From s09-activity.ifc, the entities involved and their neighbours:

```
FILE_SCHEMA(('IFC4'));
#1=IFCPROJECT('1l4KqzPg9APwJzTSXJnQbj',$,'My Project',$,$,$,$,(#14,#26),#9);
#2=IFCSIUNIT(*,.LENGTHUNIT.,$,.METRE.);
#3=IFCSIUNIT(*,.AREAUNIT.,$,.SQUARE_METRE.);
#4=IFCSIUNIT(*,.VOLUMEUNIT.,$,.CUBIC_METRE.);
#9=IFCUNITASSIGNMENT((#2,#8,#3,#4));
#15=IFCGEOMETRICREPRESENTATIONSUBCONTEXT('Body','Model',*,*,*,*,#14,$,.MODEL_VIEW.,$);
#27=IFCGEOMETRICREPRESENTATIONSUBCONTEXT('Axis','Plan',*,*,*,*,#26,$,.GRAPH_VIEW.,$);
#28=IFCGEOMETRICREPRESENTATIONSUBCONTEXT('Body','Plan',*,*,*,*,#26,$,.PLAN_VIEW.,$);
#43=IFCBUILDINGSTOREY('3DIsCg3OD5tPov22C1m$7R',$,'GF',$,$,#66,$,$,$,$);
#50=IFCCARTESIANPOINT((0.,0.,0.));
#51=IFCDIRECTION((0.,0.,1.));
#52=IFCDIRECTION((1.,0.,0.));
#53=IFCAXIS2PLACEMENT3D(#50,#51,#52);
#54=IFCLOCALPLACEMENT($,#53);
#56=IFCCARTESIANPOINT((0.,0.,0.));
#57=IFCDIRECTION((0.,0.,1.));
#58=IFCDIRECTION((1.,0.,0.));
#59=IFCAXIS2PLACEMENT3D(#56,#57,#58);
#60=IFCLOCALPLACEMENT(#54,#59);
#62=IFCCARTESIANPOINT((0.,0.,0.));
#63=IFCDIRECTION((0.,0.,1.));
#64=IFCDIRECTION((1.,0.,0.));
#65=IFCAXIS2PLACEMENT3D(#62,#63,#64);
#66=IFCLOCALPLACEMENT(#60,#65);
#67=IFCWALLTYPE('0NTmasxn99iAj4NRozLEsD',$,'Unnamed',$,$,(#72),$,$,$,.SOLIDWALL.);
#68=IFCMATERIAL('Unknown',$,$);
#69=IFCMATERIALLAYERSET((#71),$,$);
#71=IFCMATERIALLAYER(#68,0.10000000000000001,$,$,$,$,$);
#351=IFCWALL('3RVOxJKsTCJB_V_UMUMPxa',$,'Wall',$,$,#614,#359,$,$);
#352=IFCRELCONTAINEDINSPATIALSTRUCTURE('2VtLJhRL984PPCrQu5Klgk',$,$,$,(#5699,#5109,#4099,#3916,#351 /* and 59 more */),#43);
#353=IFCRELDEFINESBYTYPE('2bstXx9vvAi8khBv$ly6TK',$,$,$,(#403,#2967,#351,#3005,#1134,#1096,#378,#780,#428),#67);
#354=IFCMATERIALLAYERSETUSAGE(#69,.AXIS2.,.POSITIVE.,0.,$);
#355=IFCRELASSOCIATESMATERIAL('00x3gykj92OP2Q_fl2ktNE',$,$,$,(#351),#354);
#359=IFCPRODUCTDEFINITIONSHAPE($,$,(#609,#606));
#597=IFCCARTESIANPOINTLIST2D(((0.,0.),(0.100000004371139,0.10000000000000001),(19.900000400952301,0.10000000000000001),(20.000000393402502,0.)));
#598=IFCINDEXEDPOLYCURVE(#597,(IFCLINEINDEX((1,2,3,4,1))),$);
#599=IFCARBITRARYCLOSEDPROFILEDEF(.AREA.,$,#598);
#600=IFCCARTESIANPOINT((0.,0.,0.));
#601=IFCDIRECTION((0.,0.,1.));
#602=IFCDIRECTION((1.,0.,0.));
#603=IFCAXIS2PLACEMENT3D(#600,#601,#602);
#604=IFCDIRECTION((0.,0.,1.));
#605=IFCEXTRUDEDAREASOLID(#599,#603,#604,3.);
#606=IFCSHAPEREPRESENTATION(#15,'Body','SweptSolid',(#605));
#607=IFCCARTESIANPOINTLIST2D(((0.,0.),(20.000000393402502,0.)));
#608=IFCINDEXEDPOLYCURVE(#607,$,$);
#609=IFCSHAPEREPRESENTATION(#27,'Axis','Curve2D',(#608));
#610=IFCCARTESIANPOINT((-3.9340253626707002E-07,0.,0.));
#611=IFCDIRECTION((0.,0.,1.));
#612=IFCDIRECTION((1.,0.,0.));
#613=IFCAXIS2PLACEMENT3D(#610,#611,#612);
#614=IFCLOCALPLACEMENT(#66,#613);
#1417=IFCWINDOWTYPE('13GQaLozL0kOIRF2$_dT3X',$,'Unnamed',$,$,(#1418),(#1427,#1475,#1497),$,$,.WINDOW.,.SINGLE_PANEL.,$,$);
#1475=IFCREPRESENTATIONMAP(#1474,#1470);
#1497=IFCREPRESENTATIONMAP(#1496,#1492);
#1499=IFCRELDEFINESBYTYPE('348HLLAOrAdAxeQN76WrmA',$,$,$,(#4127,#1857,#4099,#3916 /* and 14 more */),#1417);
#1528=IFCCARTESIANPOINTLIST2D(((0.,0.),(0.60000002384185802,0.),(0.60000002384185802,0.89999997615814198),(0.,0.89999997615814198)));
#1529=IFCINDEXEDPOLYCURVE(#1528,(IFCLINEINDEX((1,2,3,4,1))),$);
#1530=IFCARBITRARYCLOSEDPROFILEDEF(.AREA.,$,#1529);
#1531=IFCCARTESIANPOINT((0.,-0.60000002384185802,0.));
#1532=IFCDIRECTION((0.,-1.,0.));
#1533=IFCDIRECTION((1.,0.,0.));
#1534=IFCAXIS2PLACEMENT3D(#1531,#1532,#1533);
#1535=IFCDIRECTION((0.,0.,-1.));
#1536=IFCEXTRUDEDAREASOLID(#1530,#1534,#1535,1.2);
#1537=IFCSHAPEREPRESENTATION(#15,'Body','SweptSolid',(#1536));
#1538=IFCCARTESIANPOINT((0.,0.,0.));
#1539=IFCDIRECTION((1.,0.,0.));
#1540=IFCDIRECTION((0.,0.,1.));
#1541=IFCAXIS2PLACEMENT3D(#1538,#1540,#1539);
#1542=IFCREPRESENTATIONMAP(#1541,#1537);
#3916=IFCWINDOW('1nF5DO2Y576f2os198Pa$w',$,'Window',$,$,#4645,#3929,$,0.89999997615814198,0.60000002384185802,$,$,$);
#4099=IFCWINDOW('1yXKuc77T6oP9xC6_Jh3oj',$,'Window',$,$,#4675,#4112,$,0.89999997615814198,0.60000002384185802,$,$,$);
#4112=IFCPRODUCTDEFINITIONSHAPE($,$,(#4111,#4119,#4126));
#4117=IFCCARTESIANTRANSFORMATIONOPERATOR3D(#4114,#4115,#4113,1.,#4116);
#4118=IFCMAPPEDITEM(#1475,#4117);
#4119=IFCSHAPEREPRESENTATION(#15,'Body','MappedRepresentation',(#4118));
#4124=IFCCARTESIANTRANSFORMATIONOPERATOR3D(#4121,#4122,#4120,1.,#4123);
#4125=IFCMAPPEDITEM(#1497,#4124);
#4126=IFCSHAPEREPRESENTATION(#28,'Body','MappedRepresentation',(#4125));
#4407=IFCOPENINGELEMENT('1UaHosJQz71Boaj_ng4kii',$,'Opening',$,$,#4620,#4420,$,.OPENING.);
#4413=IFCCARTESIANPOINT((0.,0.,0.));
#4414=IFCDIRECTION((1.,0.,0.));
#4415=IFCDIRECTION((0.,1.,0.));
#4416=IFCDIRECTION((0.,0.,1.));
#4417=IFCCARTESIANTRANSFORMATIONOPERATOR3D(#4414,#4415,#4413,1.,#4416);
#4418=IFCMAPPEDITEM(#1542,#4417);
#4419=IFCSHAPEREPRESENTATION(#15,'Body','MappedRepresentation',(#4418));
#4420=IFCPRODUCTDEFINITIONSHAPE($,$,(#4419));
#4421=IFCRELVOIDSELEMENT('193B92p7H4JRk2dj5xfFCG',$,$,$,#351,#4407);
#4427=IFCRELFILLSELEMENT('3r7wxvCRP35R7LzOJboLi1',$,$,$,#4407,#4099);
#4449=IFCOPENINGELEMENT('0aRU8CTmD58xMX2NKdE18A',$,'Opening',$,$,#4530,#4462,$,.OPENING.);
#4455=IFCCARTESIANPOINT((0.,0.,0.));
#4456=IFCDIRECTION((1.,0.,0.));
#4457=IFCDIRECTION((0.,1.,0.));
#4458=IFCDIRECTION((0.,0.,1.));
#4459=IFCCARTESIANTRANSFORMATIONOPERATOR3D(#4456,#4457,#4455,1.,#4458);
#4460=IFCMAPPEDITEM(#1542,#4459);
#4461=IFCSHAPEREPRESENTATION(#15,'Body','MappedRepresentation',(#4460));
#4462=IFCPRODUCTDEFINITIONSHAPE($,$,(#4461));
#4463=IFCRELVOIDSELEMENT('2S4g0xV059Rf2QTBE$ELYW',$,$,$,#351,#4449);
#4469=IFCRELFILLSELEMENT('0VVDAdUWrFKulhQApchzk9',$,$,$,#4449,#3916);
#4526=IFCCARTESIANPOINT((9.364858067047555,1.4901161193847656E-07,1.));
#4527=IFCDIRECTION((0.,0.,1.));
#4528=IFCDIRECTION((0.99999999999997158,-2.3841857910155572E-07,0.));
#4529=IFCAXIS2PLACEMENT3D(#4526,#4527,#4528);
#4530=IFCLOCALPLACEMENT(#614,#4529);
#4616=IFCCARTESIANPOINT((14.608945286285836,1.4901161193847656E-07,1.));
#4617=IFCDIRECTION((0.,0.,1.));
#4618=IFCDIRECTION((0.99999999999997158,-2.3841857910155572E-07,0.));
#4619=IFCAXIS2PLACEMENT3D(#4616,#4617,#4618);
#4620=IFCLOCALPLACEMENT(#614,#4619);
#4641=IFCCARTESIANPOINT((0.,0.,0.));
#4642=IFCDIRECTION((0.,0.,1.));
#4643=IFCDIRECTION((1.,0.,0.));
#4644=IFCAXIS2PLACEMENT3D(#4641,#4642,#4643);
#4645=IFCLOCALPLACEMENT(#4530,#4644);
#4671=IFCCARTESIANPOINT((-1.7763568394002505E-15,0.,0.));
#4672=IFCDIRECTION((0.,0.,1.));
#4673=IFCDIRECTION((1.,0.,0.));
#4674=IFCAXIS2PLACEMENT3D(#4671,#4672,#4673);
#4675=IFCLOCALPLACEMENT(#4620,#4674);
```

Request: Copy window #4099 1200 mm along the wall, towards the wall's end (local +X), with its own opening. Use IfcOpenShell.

```python
import ifcopenshell
import ifcopenshell.api.feature
import ifcopenshell.api.geometry
import ifcopenshell.api.root
import ifcopenshell.geom
import ifcopenshell.util.element
import ifcopenshell.util.placement
import ifcopenshell.util.shape
import ifcopenshell.util.unit

model = ifcopenshell.open("s09-activity.ifc")
unit_scale = ifcopenshell.util.unit.calculate_unit_scale(model)
settings = ifcopenshell.geom.settings()


def volume(element):
    """Net volume in cubic metres, openings subtracted."""
    shape = ifcopenshell.geom.create_shape(settings, element)
    return ifcopenshell.util.shape.get_volume(shape.geometry)


window = model.by_guid("1yXKuc77T6oP9xC6_Jh3oj")
opening = window.FillsVoids[0].RelatingOpeningElement
wall = opening.VoidsElements[0].RelatingBuildingElement
before = volume(wall)
shift = ifcopenshell.util.placement.get_local_placement(wall.ObjectPlacement)[:3, 0] * 1.2 / unit_scale

# copy_class copies the void relationship, type, container and properties, but no geometry.
new_opening = ifcopenshell.api.root.copy_class(model, product=opening)
new_opening.Representation = ifcopenshell.util.element.copy_deep(
    model, opening.Representation, exclude=["IfcGeometricRepresentationContext", "IfcRepresentationMap"]
)
new_window = ifcopenshell.api.root.copy_class(model, product=window)
new_window.Representation = ifcopenshell.util.element.copy_deep(
    model, window.Representation, exclude=["IfcGeometricRepresentationContext", "IfcRepresentationMap"]
)
ifcopenshell.api.feature.add_filling(model, opening=new_opening, element=new_window)

for old, new in ((opening, new_opening), (window, new_window)):
    matrix = ifcopenshell.util.placement.get_local_placement(old.ObjectPlacement)
    matrix[:3, 3] += shift
    ifcopenshell.api.geometry.edit_object_placement(model, product=new, matrix=matrix, is_si=False)

after = volume(wall)

print(f"wall volume {before:.3f} -> {after:.3f} m3")

model.write("s09-activity_edited.ifc")
```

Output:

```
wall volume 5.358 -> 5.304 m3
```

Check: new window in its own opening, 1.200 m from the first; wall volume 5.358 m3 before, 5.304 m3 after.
